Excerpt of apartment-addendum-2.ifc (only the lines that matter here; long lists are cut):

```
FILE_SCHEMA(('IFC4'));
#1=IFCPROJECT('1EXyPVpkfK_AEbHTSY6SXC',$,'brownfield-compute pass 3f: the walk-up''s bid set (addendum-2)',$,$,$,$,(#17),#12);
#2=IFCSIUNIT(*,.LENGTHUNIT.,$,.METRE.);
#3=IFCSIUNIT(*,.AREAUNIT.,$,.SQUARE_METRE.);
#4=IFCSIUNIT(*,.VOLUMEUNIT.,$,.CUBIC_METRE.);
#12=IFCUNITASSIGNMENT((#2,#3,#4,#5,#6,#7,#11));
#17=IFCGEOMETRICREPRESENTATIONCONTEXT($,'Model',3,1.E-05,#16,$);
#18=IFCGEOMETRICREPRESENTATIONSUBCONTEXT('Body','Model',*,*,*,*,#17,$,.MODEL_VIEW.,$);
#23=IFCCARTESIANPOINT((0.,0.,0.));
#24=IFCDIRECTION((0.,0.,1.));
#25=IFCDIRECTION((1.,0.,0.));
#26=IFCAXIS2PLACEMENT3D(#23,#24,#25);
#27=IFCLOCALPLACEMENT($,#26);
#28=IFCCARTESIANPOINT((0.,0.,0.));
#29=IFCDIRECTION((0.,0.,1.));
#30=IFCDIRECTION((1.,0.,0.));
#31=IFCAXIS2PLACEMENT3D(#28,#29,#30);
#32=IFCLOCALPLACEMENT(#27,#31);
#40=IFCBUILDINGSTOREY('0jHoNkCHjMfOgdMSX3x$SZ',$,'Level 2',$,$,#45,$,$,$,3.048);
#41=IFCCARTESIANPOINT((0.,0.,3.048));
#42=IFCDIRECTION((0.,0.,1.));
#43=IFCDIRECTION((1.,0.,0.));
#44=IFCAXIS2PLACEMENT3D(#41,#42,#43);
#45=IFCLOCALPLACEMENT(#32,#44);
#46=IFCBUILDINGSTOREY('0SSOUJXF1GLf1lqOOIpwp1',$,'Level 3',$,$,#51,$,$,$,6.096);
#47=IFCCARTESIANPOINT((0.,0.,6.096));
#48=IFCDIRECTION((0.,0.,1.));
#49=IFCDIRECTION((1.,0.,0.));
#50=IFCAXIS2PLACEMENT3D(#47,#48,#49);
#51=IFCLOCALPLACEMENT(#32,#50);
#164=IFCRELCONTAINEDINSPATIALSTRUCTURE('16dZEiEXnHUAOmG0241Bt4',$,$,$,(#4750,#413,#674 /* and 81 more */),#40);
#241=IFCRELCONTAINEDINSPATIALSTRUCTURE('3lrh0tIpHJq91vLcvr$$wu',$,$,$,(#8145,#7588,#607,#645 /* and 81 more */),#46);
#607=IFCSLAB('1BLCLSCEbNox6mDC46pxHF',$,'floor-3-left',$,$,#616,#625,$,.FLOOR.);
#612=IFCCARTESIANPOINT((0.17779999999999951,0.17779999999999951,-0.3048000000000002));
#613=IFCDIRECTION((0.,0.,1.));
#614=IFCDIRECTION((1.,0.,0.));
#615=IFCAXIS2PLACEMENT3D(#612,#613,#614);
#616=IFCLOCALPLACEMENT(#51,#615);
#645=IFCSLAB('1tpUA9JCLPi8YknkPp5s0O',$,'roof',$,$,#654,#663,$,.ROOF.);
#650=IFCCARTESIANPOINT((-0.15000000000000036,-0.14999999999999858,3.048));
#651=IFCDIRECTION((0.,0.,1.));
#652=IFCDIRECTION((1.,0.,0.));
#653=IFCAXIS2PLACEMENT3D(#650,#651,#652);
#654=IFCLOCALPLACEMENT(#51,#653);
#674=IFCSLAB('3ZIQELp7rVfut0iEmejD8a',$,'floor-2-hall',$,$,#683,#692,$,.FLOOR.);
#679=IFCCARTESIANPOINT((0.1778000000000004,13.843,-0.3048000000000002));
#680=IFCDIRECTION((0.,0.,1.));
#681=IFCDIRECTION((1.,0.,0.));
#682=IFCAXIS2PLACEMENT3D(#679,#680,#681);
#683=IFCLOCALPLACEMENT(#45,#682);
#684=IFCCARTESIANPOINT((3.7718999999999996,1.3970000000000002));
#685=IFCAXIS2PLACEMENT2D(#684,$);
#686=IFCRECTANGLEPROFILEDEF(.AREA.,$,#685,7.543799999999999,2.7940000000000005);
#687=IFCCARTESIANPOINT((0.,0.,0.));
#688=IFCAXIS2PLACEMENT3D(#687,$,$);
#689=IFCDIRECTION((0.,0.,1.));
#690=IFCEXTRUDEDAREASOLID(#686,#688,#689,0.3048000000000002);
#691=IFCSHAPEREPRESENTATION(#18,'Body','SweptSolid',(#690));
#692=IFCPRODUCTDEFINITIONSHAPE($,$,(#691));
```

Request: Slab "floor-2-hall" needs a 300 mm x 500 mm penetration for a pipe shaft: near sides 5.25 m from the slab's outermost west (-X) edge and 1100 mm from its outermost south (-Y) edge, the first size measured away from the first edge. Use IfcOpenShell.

```python
import numpy as np
import ifcopenshell
import ifcopenshell.api.feature
import ifcopenshell.api.geometry
import ifcopenshell.api.root
import ifcopenshell.geom
import ifcopenshell.util.placement
import ifcopenshell.util.representation
import ifcopenshell.util.shape
import ifcopenshell.util.unit

model = ifcopenshell.open("apartment-addendum-2.ifc")
unit_scale = ifcopenshell.util.unit.calculate_unit_scale(model)
settings = ifcopenshell.geom.settings()


def volume(element):
    """Net volume in cubic metres, openings subtracted."""
    shape = ifcopenshell.geom.create_shape(settings, element)
    return ifcopenshell.util.shape.get_volume(shape.geometry)


slab = model.by_guid("3ZIQELp7rVfut0iEmejD8a")
before = volume(slab)

# Extent in the slab's own axes, in metres. The edges named are its -X and -Y sides.
slab_shape = ifcopenshell.geom.create_shape(settings, slab)
vertices = ifcopenshell.util.shape.get_vertices(slab_shape.geometry)
x_min, y_min, bottom = vertices.min(axis=0)
top = vertices[:, 2].max()

opening = ifcopenshell.api.root.create_entity(model, ifc_class="IfcOpeningElement", name="Pipe shaft opening", predefined_type="OPENING")
context = ifcopenshell.util.representation.get_context(model, "Model", "Body", "MODEL_VIEW")
width, depth = 0.3, 0.5
outline = [(0.0, 0.0), (width, 0.0), (width, depth), (0.0, depth), (0.0, 0.0)]
# Overshoot both faces by 50 mm so the cut is clean.
shape = ifcopenshell.api.geometry.add_slab_representation(
    model, context=context, depth=top - bottom + 0.1, polyline=outline
)
ifcopenshell.api.geometry.assign_representation(model, product=opening, representation=shape)

matrix = ifcopenshell.util.placement.get_local_placement(slab.ObjectPlacement)
matrix[:, 3] = matrix @ np.append(np.array([x_min + 5.25, y_min + 1.1, bottom - 0.05]) / unit_scale, 1.0)
ifcopenshell.api.geometry.edit_object_placement(model, product=opening, matrix=matrix, is_si=False)
ifcopenshell.api.feature.add_feature(model, feature=opening, element=slab)

after = volume(slab)

print(f"slab volume {before:.3f} -> {after:.3f} m3")

model.write("apartment-addendum-2_edited.ifc")
```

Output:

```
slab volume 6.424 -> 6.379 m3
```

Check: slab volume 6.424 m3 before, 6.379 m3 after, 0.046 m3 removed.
